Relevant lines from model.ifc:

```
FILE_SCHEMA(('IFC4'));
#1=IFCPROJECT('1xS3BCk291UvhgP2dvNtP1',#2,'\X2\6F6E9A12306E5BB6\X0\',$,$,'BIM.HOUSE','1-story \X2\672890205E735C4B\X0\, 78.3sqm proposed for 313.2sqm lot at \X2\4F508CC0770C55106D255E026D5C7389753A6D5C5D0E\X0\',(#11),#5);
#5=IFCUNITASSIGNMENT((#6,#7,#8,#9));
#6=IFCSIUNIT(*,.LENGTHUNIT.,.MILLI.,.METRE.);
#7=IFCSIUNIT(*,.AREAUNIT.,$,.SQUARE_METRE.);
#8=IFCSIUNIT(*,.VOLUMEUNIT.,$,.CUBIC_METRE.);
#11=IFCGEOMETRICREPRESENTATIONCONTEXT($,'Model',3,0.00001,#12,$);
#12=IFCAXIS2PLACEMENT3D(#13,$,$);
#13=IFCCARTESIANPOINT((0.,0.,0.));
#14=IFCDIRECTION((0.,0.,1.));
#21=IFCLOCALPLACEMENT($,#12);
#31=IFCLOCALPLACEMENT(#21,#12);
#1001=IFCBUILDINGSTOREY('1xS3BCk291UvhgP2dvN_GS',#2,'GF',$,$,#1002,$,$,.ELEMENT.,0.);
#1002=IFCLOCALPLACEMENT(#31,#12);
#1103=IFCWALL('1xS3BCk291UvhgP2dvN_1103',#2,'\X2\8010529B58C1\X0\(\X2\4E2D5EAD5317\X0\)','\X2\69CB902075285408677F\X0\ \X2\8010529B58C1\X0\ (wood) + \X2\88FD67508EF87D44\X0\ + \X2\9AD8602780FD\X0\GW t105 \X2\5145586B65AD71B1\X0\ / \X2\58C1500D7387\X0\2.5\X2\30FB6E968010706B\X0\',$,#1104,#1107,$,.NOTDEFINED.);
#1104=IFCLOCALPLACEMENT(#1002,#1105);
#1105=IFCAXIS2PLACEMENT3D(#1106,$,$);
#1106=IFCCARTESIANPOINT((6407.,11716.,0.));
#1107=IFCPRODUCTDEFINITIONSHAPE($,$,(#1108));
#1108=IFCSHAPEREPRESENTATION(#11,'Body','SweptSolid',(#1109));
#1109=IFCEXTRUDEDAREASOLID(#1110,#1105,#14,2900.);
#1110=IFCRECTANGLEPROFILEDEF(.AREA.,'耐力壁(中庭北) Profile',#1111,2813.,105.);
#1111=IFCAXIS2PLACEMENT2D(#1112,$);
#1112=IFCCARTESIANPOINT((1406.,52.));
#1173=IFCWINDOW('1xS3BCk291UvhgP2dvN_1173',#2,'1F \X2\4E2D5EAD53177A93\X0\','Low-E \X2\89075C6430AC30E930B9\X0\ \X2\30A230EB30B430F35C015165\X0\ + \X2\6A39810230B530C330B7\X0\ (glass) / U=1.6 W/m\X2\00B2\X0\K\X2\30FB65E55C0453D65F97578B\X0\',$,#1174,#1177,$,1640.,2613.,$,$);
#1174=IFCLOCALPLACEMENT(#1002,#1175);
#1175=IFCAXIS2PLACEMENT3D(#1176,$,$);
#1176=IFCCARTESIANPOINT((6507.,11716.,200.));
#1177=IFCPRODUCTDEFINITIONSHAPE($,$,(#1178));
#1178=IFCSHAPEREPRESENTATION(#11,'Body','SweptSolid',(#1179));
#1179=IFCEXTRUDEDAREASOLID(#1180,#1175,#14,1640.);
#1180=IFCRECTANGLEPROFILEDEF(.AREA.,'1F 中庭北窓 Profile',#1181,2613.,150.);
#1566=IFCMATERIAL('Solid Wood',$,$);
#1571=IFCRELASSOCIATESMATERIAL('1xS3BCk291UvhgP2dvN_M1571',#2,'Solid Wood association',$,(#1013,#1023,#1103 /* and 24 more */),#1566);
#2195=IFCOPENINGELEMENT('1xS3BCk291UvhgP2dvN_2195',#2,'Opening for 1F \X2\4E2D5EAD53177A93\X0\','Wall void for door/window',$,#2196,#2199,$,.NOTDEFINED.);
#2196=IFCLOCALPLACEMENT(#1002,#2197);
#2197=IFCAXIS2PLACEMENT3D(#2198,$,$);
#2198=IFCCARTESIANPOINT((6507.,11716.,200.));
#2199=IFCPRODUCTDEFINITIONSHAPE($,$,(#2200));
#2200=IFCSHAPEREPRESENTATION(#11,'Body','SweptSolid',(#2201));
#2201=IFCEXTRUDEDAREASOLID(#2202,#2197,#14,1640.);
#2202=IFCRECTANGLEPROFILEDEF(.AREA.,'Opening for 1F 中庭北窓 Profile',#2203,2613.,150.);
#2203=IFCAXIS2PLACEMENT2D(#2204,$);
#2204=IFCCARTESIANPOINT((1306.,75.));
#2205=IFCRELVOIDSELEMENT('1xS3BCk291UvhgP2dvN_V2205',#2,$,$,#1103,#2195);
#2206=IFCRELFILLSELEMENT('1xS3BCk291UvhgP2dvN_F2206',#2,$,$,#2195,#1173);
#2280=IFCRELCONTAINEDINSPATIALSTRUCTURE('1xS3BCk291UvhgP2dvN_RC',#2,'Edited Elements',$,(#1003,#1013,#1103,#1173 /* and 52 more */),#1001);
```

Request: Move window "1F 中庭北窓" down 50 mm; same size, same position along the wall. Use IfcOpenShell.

```python
import numpy as np
import ifcopenshell
import ifcopenshell.api.geometry
import ifcopenshell.util.placement
import ifcopenshell.util.unit

model = ifcopenshell.open("model.ifc")
unit_scale = ifcopenshell.util.unit.calculate_unit_scale(model)

window = model.by_id(1173)
opening = window.FillsVoids[0].RelatingOpeningElement
dz = -50.0

shift = np.array([0.0, 0.0, dz])
# The window is not placed relative to its opening, so move both.
for product in (opening, window):
    matrix = ifcopenshell.util.placement.get_local_placement(product.ObjectPlacement)
    matrix[:3, 3] += shift
    ifcopenshell.api.geometry.edit_object_placement(model, product=product, matrix=matrix, is_si=False)

print(f"moved by {dz * unit_scale:+.3f} m")

model.write("model-out.ifc")
```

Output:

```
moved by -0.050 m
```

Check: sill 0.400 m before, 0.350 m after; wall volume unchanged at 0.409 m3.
